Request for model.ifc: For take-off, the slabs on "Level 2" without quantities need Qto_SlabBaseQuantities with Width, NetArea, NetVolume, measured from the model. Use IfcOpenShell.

First a look at what the model holds.

```python
import ifcopenshell
import ifcopenshell.util.element
import ifcopenshell.util.unit

model = ifcopenshell.open("model.ifc")
print(model.schema)
for unit_type in ("LENGTHUNIT", "AREAUNIT", "VOLUMEUNIT"):
    print(unit_type, ifcopenshell.util.unit.calculate_unit_scale(model, unit_type))
storey = next(s for s in model.by_type("IfcBuildingStorey") if s.Name == "Level 2")
slabs = [e for e in ifcopenshell.util.element.get_decomposition(storey) if e.is_a("IfcSlab")]
for e in sorted(slabs, key=lambda e: e.id()):
    print(e.id(), e.is_a(), e.Name, list(ifcopenshell.util.element.get_psets(e, qtos_only=True)), sep=" | ")
```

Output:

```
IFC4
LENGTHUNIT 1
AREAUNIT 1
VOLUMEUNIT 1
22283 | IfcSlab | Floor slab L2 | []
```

```python
import ifcopenshell
import ifcopenshell.api.pset
import ifcopenshell.geom
import ifcopenshell.util.element
import ifcopenshell.util.shape
import ifcopenshell.util.unit

model = ifcopenshell.open("model.ifc")
unit_scale = ifcopenshell.util.unit.calculate_unit_scale(model)
area_scale = ifcopenshell.util.unit.calculate_unit_scale(model, "AREAUNIT")
volume_scale = ifcopenshell.util.unit.calculate_unit_scale(model, "VOLUMEUNIT")
settings = ifcopenshell.geom.settings()

storey = next(s for s in model.by_type("IfcBuildingStorey") if s.Name == "Level 2")
slabs = [e for e in ifcopenshell.util.element.get_decomposition(storey) if e.is_a("IfcSlab")]

for e in sorted(slabs, key=lambda e: e.id()):
    if ifcopenshell.util.element.get_psets(e, qtos_only=True, should_inherit=False):
        continue
    # Geometry comes back in metres, in the element's own axes.
    shape = ifcopenshell.geom.create_shape(settings, e)
    values = {
        "Width": ifcopenshell.util.shape.get_z(shape.geometry) / unit_scale,
        "NetArea": ifcopenshell.util.shape.get_footprint_area(shape.geometry) / area_scale,
        "NetVolume": ifcopenshell.util.shape.get_volume(shape.geometry) / volume_scale,
    }
    qto = ifcopenshell.api.pset.add_qto(model, product=e, name="Qto_SlabBaseQuantities")
    ifcopenshell.api.pset.edit_qto(model, qto=qto, properties=values)
    print(e.id(), {k: round(v, 3) for k, v in values.items()})

model.write("model_v2.ifc")
```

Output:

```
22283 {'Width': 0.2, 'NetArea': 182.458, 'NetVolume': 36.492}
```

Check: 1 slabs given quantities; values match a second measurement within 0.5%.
